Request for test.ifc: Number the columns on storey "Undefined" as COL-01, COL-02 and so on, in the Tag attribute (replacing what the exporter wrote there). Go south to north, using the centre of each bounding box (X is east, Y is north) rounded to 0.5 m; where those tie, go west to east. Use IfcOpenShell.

First a look at what the model holds.

```python
import ifcopenshell
import ifcopenshell.util.element
import ifcopenshell.util.placement

model = ifcopenshell.open("test.ifc")
print(model.schema)
storey = next(s for s in model.by_type("IfcBuildingStorey") if s.Name == "Undefined")
columns = [e for e in ifcopenshell.util.element.get_decomposition(storey) if e.is_a("IfcColumn")]
for e in sorted(columns, key=lambda e: e.id()):
    origin = ifcopenshell.util.placement.get_local_placement(e.ObjectPlacement)[:3, 3]
    print(e.id(), e.Tag, e.Name, origin.round(2) + 0.0, sep=" | ")
```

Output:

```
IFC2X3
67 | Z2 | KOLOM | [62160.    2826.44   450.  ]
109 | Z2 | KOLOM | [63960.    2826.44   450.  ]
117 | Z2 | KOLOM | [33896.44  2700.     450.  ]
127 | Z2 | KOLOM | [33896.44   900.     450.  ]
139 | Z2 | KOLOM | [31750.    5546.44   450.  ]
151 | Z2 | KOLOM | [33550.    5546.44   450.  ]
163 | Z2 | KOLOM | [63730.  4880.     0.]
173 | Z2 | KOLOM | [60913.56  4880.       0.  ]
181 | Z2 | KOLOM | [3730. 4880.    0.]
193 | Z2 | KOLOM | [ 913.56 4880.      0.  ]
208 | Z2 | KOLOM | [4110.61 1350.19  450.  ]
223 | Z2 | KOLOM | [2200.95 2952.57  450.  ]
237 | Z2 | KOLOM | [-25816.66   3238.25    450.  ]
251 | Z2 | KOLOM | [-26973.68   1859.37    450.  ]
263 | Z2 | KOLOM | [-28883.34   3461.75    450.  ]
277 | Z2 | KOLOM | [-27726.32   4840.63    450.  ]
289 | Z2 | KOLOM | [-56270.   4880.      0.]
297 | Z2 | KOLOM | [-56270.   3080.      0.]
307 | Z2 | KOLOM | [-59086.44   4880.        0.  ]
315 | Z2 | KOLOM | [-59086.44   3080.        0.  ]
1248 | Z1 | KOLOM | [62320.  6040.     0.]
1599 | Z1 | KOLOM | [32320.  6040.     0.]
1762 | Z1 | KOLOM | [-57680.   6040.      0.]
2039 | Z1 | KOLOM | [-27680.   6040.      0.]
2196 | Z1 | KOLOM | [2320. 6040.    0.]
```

```python
import ifcopenshell
import ifcopenshell.geom
import ifcopenshell.util.element
import ifcopenshell.util.shape

model = ifcopenshell.open("test.ifc")
settings = ifcopenshell.geom.settings()
settings.set("use-world-coords", True)


def centre(element):
    shape = ifcopenshell.geom.create_shape(settings, element)
    return ifcopenshell.util.shape.get_bbox_centroid(shape.geometry)


storey = next(s for s in model.by_type("IfcBuildingStorey") if s.Name == "Undefined")
columns = [e for e in ifcopenshell.util.element.get_decomposition(storey) if e.is_a("IfcColumn")]

# Insertion points can sit at a corner or the storey origin, so sort by the geometry (in metres).
centres = {e: centre(e) for e in columns}
columns.sort(key=lambda e: (round(centres[e][1] / 0.5), centres[e][0]))

for i, e in enumerate(columns, start=1):
    number = f"COL-{i:02d}"
    e.Tag = number
    print(e.id(), number)

model.write("test_v2.ifc")
```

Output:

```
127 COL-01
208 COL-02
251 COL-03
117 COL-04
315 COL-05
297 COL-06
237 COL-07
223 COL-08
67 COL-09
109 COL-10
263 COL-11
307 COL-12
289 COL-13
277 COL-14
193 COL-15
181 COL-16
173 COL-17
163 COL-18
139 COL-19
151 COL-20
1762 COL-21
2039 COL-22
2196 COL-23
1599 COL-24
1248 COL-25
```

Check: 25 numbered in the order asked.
